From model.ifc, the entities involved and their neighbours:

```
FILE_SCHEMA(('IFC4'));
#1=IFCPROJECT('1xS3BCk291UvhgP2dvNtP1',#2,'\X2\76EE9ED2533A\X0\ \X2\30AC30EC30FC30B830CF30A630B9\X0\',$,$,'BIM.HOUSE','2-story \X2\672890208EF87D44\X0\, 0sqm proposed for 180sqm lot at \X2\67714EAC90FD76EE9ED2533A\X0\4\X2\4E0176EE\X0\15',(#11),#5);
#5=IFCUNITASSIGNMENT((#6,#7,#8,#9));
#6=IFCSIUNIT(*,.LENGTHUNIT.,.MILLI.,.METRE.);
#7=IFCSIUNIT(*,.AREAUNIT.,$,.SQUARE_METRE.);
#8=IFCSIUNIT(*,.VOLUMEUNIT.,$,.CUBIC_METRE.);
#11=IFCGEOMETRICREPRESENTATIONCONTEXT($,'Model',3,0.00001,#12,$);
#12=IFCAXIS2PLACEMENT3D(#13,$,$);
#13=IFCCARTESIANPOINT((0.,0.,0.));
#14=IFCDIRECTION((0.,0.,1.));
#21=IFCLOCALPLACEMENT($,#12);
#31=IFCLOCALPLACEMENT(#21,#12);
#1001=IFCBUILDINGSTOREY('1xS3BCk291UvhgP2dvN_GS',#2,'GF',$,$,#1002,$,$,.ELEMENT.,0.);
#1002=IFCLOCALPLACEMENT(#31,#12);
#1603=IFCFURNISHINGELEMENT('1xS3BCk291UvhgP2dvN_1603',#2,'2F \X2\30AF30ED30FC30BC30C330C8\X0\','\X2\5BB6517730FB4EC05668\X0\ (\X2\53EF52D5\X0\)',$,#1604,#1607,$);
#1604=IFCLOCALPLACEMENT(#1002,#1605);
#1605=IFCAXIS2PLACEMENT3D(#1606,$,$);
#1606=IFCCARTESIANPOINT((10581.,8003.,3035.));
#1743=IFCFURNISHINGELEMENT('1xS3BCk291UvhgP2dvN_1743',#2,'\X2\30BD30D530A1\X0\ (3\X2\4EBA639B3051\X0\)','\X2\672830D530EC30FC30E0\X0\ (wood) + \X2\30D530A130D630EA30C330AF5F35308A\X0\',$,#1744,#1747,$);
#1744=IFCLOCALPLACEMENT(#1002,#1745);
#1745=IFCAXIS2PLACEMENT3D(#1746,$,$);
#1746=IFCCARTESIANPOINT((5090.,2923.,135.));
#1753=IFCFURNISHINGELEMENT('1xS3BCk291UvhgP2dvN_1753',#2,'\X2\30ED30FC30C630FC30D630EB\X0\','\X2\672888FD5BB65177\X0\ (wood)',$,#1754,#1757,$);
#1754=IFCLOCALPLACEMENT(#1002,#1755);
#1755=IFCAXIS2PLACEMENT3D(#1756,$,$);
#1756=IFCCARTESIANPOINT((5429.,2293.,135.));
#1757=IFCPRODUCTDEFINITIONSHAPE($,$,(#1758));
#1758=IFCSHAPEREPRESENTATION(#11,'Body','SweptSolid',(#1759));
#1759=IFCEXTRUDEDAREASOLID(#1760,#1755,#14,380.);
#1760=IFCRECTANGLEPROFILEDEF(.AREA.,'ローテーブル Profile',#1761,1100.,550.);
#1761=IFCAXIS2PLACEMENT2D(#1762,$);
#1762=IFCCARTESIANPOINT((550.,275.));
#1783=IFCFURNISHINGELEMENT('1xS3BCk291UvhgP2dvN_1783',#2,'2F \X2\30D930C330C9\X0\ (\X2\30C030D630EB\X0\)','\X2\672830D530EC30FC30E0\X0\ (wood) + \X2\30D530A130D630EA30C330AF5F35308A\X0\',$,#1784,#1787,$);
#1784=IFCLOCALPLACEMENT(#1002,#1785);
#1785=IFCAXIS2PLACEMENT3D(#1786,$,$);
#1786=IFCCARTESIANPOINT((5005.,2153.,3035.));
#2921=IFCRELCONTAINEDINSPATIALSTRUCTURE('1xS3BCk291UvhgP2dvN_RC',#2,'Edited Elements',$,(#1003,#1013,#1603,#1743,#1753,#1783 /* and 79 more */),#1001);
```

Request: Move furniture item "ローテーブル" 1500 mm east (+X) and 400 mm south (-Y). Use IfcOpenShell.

```python
import ifcopenshell
import ifcopenshell.api.geometry
import ifcopenshell.util.placement

model = ifcopenshell.open("model.ifc")

item = model.by_id(1753)
matrix = ifcopenshell.util.placement.get_local_placement(item.ObjectPlacement)
matrix[0, 3] += 1500.0
matrix[1, 3] -= 400.0
ifcopenshell.api.geometry.edit_object_placement(model, product=item, matrix=matrix, is_si=False)

print(ifcopenshell.util.placement.get_local_placement(item.ObjectPlacement).round(3) + 0.0)

model.write("model_edited.ifc")
```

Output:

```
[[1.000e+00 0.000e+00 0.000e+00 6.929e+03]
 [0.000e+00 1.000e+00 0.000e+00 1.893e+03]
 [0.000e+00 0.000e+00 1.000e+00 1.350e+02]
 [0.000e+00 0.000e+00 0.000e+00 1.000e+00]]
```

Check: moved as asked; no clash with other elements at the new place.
